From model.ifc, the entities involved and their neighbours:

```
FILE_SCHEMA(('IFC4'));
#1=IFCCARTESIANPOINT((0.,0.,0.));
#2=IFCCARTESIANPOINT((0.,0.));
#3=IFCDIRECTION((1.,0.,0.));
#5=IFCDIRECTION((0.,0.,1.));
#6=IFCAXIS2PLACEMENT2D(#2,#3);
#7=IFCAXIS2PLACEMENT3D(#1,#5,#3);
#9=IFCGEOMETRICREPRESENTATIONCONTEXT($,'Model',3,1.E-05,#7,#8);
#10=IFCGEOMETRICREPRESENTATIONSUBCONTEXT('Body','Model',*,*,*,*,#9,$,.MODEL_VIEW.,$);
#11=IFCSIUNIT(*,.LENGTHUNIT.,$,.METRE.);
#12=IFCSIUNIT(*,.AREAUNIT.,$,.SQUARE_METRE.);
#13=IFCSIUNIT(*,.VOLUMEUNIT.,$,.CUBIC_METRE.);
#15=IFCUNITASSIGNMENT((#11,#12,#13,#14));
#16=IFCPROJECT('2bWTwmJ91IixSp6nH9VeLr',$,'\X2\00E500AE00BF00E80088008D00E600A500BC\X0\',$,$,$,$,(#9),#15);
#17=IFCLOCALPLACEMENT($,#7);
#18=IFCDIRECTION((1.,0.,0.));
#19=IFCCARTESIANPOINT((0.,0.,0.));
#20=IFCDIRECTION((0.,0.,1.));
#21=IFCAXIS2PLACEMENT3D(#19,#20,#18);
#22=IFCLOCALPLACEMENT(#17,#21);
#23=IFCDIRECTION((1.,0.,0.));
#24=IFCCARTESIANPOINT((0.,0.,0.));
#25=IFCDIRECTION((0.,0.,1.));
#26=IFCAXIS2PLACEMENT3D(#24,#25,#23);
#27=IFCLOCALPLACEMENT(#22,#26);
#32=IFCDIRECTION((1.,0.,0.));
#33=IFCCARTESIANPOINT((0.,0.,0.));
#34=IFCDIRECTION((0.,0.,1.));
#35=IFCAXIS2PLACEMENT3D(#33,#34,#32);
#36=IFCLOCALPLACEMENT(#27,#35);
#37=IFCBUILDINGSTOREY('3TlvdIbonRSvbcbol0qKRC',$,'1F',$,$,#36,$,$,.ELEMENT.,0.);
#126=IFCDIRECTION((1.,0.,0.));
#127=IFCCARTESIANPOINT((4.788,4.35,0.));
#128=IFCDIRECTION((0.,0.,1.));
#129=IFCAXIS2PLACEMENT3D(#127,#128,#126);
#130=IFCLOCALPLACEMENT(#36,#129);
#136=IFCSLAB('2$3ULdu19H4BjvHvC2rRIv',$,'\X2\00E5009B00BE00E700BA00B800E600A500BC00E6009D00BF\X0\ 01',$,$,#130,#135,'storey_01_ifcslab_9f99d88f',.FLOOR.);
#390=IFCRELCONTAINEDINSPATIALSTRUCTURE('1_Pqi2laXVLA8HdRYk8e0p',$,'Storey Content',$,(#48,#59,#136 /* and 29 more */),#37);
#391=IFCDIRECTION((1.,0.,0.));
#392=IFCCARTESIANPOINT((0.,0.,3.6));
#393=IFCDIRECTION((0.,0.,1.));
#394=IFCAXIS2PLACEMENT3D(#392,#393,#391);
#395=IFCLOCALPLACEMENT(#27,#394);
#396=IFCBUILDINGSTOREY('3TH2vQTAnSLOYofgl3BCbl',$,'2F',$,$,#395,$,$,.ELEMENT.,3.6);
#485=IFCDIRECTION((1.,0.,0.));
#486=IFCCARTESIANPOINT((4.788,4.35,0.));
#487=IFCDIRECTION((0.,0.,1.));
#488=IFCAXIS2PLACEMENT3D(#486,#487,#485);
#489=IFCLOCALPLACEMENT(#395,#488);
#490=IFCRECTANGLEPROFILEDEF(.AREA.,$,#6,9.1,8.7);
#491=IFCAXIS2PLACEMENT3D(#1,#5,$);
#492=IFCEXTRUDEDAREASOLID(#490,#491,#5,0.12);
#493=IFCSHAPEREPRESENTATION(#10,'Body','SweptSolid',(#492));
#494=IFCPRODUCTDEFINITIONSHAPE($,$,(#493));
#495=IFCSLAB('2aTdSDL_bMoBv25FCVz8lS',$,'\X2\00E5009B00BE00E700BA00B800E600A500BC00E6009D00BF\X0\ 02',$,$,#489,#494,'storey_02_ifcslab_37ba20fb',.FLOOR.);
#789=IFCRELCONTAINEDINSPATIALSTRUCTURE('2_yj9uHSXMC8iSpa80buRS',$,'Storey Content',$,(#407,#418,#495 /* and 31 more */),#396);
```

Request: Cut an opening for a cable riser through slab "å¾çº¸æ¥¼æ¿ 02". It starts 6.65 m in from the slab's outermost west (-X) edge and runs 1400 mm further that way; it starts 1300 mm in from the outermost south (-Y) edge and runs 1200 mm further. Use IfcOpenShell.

```python
import numpy as np
import ifcopenshell
import ifcopenshell.api.feature
import ifcopenshell.api.geometry
import ifcopenshell.api.root
import ifcopenshell.geom
import ifcopenshell.util.placement
import ifcopenshell.util.representation
import ifcopenshell.util.shape
import ifcopenshell.util.unit

model = ifcopenshell.open("model.ifc")
unit_scale = ifcopenshell.util.unit.calculate_unit_scale(model)
settings = ifcopenshell.geom.settings()


def volume(element):
    """Net volume in cubic metres, openings subtracted."""
    shape = ifcopenshell.geom.create_shape(settings, element)
    return ifcopenshell.util.shape.get_volume(shape.geometry)


slab = model.by_guid("2aTdSDL_bMoBv25FCVz8lS")
before = volume(slab)

# Extent in the slab's own axes, in metres. The edges named are its -X and -Y sides.
slab_shape = ifcopenshell.geom.create_shape(settings, slab)
vertices = ifcopenshell.util.shape.get_vertices(slab_shape.geometry)
x_min, y_min, bottom = vertices.min(axis=0)
top = vertices[:, 2].max()

opening = ifcopenshell.api.root.create_entity(model, ifc_class="IfcOpeningElement", name="Cable riser opening", predefined_type="OPENING")
context = ifcopenshell.util.representation.get_context(model, "Model", "Body", "MODEL_VIEW")
width, depth = 1.4, 1.2
outline = [(0.0, 0.0), (width, 0.0), (width, depth), (0.0, depth), (0.0, 0.0)]
# Overshoot both faces by 50 mm so the cut is clean.
shape = ifcopenshell.api.geometry.add_slab_representation(
    model, context=context, depth=top - bottom + 0.1, polyline=outline
)
ifcopenshell.api.geometry.assign_representation(model, product=opening, representation=shape)

matrix = ifcopenshell.util.placement.get_local_placement(slab.ObjectPlacement)
matrix[:, 3] = matrix @ np.append(np.array([x_min + 6.65, y_min + 1.3, bottom - 0.05]) / unit_scale, 1.0)
ifcopenshell.api.geometry.edit_object_placement(model, product=opening, matrix=matrix, is_si=False)
ifcopenshell.api.feature.add_feature(model, feature=opening, element=slab)

after = volume(slab)

print(f"slab volume {before:.3f} -> {after:.3f} m3")

model.write("model_updated.ifc")
```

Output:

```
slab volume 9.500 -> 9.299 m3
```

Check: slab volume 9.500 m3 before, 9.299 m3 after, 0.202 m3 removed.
